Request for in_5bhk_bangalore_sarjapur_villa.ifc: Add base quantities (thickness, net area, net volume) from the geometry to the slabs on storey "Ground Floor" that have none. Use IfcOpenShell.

First a look at what the model holds.

```python
import ifcopenshell
import ifcopenshell.util.element
import ifcopenshell.util.unit

model = ifcopenshell.open("in_5bhk_bangalore_sarjapur_villa.ifc")
print(model.schema)
for unit_type in ("LENGTHUNIT", "AREAUNIT", "VOLUMEUNIT"):
    print(unit_type, ifcopenshell.util.unit.calculate_unit_scale(model, unit_type))
storey = next(s for s in model.by_type("IfcBuildingStorey") if s.Name == "Ground Floor")
slabs = [e for e in ifcopenshell.util.element.get_decomposition(storey) if e.is_a("IfcSlab")]
for e in sorted(slabs, key=lambda e: e.id()):
    print(e.id(), e.is_a(), e.Name, list(ifcopenshell.util.element.get_psets(e, qtos_only=True)), sep=" | ")
```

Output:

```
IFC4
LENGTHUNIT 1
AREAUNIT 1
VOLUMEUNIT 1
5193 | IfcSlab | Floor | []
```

```python
import ifcopenshell
import ifcopenshell.api.pset
import ifcopenshell.geom
import ifcopenshell.util.element
import ifcopenshell.util.shape
import ifcopenshell.util.unit

model = ifcopenshell.open("in_5bhk_bangalore_sarjapur_villa.ifc")
unit_scale = ifcopenshell.util.unit.calculate_unit_scale(model)
area_scale = ifcopenshell.util.unit.calculate_unit_scale(model, "AREAUNIT")
volume_scale = ifcopenshell.util.unit.calculate_unit_scale(model, "VOLUMEUNIT")
settings = ifcopenshell.geom.settings()

storey = next(s for s in model.by_type("IfcBuildingStorey") if s.Name == "Ground Floor")
slabs = [e for e in ifcopenshell.util.element.get_decomposition(storey) if e.is_a("IfcSlab")]

for e in sorted(slabs, key=lambda e: e.id()):
    if ifcopenshell.util.element.get_psets(e, qtos_only=True, should_inherit=False):
        continue
    # Geometry comes back in metres, in the element's own axes.
    shape = ifcopenshell.geom.create_shape(settings, e)
    values = {
        "Width": ifcopenshell.util.shape.get_z(shape.geometry) / unit_scale,
        "NetArea": ifcopenshell.util.shape.get_footprint_area(shape.geometry) / area_scale,
        "NetVolume": ifcopenshell.util.shape.get_volume(shape.geometry) / volume_scale,
    }
    qto = ifcopenshell.api.pset.add_qto(model, product=e, name="Qto_SlabBaseQuantities")
    ifcopenshell.api.pset.edit_qto(model, qto=qto, properties=values)
    print(e.id(), {k: round(v, 3) for k, v in values.items()})

model.write("in_5bhk_bangalore_sarjapur_villa-out.ifc")
```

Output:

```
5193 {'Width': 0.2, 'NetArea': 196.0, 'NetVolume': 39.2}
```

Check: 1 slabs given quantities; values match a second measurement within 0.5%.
